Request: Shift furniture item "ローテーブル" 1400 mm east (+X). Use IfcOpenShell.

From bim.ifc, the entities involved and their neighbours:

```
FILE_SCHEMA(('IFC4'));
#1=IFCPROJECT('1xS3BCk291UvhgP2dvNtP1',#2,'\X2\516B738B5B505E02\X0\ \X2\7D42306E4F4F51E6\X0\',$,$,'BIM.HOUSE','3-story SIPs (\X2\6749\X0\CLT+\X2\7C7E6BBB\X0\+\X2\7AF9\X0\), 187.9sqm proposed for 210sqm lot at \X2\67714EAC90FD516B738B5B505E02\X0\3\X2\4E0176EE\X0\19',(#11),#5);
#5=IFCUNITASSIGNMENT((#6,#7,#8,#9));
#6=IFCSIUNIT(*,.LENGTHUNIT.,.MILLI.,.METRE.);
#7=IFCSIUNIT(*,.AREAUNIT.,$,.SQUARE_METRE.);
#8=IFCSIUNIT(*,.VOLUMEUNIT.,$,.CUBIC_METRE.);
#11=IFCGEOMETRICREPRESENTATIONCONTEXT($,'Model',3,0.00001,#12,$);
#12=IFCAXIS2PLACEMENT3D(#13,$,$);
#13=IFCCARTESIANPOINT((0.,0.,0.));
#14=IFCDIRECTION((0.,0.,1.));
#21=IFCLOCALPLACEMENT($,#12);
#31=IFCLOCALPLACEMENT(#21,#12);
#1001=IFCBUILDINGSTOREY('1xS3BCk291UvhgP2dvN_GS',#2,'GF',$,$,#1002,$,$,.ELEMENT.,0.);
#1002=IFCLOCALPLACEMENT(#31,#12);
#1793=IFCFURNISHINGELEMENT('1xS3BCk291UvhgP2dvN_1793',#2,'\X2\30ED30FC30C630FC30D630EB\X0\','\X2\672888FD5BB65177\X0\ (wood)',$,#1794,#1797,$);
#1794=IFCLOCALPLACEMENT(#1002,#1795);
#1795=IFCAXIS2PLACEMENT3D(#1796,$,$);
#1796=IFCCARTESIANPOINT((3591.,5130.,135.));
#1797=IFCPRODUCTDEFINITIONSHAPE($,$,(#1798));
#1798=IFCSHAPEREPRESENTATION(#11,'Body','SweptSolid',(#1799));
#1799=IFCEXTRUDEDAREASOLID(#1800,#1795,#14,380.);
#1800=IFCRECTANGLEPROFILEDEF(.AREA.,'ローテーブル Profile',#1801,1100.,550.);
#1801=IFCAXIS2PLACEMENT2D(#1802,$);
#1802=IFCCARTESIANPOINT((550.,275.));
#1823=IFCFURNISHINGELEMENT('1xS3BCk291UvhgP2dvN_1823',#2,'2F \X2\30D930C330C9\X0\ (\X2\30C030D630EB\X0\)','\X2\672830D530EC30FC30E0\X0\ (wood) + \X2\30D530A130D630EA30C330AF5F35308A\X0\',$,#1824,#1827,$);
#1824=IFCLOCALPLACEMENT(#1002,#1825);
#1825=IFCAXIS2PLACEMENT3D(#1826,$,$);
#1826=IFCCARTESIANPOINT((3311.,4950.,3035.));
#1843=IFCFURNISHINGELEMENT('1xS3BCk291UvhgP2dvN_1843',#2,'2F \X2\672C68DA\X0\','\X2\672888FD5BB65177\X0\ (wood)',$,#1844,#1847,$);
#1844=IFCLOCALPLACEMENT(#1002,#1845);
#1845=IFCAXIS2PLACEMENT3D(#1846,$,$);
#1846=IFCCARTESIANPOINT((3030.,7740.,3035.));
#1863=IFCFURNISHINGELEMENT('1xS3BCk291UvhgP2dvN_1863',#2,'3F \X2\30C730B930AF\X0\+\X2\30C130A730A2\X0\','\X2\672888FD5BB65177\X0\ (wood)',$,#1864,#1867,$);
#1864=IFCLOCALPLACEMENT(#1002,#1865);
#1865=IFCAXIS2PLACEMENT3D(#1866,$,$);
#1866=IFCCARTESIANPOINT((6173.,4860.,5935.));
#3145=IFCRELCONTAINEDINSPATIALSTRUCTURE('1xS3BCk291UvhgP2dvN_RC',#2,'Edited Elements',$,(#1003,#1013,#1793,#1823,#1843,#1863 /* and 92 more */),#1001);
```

```python
import ifcopenshell
import ifcopenshell.api.geometry
import ifcopenshell.util.placement

model = ifcopenshell.open("bim.ifc")

item = model.by_id(1793)
matrix = ifcopenshell.util.placement.get_local_placement(item.ObjectPlacement)
matrix[0, 3] += 1400.0
ifcopenshell.api.geometry.edit_object_placement(model, product=item, matrix=matrix, is_si=False)

print(ifcopenshell.util.placement.get_local_placement(item.ObjectPlacement).round(3) + 0.0)

model.write("bim_updated.ifc")
```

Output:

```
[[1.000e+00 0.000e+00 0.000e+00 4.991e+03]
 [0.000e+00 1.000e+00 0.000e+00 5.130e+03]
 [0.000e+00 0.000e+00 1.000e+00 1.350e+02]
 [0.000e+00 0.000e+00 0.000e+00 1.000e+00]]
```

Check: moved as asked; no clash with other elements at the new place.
